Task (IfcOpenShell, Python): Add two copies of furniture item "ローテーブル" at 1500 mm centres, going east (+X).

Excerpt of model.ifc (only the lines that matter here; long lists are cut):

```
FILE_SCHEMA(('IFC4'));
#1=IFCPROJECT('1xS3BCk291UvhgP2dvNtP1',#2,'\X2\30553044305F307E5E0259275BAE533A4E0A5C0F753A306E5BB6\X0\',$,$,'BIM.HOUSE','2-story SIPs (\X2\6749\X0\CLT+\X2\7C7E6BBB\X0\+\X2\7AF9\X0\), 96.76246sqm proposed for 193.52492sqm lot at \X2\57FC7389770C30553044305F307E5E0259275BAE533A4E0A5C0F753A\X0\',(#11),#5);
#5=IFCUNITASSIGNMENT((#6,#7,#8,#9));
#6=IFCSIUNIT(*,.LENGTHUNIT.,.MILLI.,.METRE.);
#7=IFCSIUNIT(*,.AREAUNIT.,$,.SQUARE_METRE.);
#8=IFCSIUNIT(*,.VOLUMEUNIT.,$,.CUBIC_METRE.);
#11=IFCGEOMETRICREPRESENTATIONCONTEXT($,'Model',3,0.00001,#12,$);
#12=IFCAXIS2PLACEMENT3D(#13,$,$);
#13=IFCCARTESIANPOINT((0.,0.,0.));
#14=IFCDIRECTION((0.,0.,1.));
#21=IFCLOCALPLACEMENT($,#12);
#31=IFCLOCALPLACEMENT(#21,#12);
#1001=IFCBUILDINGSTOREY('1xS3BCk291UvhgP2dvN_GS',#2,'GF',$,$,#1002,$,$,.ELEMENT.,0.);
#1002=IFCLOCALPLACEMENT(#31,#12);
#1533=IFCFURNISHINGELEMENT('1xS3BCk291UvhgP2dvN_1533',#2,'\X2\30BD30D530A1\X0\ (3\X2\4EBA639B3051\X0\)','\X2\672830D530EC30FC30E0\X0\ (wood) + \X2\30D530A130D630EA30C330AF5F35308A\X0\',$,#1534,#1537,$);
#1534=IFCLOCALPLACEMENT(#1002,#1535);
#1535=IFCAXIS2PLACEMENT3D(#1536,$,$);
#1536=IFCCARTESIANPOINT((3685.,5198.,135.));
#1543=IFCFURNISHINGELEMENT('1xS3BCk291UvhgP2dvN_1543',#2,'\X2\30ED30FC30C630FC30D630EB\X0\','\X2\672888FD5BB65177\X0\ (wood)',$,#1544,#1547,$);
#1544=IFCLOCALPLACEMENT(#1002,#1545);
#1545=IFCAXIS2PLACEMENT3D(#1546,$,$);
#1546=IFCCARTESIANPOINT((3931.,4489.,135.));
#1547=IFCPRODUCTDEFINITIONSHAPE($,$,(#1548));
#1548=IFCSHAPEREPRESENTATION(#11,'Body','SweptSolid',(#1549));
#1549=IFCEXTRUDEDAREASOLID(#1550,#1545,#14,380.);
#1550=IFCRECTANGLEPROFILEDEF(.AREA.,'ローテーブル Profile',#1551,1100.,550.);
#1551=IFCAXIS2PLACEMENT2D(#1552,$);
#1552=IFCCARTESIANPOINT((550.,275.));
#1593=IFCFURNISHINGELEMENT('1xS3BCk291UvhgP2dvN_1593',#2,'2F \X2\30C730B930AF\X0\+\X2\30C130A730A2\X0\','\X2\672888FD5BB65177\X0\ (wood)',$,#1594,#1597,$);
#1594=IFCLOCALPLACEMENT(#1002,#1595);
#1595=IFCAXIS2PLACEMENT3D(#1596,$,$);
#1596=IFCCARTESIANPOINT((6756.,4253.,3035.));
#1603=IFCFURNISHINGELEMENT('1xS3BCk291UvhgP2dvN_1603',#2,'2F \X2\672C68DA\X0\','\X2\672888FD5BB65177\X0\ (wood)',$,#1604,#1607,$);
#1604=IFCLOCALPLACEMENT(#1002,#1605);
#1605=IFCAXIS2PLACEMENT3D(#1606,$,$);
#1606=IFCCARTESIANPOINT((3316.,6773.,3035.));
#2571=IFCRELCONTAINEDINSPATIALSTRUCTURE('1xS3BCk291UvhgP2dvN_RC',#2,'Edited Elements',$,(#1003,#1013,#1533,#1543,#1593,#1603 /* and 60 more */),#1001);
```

```python
import numpy as np
import ifcopenshell
import ifcopenshell.api.geometry
import ifcopenshell.api.root
import ifcopenshell.util.element
import ifcopenshell.util.placement
import ifcopenshell.util.unit

model = ifcopenshell.open("model.ifc")
unit_scale = ifcopenshell.util.unit.calculate_unit_scale(model)


def reuse_history(source, copy):
    """copy_class also copies each property set's owner history, people and application; keep the originals."""
    for rel in copy.IsDefinedBy:
        if rel.is_a("IfcRelDefinesByProperties") and (history := rel.RelatingPropertyDefinition.OwnerHistory):
            rel.RelatingPropertyDefinition.OwnerHistory = source.OwnerHistory
            ifcopenshell.util.element.remove_deep2(model, history)


source = model.by_guid("1xS3BCk291UvhgP2dvN_1543")
base = ifcopenshell.util.placement.get_local_placement(source.ObjectPlacement)
step = np.array([1.0, 0.0, 0.0]) * 1.5 / unit_scale

for i in range(1, 3):
    copy = ifcopenshell.api.root.copy_class(model, product=source)
    copy.Representation = ifcopenshell.util.element.copy_deep(
        model, source.Representation, exclude=["IfcGeometricRepresentationContext", "IfcRepresentationMap"]
    )
    reuse_history(source, copy)
    matrix = base.copy()
    matrix[:3, 3] += i * step
    print("added at", matrix[:3, 3].round(3) + 0.0)
    ifcopenshell.api.geometry.edit_object_placement(model, product=copy, matrix=matrix, is_si=False)

model.write("model-out.ifc")
```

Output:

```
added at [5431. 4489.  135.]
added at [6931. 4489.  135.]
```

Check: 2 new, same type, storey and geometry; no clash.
